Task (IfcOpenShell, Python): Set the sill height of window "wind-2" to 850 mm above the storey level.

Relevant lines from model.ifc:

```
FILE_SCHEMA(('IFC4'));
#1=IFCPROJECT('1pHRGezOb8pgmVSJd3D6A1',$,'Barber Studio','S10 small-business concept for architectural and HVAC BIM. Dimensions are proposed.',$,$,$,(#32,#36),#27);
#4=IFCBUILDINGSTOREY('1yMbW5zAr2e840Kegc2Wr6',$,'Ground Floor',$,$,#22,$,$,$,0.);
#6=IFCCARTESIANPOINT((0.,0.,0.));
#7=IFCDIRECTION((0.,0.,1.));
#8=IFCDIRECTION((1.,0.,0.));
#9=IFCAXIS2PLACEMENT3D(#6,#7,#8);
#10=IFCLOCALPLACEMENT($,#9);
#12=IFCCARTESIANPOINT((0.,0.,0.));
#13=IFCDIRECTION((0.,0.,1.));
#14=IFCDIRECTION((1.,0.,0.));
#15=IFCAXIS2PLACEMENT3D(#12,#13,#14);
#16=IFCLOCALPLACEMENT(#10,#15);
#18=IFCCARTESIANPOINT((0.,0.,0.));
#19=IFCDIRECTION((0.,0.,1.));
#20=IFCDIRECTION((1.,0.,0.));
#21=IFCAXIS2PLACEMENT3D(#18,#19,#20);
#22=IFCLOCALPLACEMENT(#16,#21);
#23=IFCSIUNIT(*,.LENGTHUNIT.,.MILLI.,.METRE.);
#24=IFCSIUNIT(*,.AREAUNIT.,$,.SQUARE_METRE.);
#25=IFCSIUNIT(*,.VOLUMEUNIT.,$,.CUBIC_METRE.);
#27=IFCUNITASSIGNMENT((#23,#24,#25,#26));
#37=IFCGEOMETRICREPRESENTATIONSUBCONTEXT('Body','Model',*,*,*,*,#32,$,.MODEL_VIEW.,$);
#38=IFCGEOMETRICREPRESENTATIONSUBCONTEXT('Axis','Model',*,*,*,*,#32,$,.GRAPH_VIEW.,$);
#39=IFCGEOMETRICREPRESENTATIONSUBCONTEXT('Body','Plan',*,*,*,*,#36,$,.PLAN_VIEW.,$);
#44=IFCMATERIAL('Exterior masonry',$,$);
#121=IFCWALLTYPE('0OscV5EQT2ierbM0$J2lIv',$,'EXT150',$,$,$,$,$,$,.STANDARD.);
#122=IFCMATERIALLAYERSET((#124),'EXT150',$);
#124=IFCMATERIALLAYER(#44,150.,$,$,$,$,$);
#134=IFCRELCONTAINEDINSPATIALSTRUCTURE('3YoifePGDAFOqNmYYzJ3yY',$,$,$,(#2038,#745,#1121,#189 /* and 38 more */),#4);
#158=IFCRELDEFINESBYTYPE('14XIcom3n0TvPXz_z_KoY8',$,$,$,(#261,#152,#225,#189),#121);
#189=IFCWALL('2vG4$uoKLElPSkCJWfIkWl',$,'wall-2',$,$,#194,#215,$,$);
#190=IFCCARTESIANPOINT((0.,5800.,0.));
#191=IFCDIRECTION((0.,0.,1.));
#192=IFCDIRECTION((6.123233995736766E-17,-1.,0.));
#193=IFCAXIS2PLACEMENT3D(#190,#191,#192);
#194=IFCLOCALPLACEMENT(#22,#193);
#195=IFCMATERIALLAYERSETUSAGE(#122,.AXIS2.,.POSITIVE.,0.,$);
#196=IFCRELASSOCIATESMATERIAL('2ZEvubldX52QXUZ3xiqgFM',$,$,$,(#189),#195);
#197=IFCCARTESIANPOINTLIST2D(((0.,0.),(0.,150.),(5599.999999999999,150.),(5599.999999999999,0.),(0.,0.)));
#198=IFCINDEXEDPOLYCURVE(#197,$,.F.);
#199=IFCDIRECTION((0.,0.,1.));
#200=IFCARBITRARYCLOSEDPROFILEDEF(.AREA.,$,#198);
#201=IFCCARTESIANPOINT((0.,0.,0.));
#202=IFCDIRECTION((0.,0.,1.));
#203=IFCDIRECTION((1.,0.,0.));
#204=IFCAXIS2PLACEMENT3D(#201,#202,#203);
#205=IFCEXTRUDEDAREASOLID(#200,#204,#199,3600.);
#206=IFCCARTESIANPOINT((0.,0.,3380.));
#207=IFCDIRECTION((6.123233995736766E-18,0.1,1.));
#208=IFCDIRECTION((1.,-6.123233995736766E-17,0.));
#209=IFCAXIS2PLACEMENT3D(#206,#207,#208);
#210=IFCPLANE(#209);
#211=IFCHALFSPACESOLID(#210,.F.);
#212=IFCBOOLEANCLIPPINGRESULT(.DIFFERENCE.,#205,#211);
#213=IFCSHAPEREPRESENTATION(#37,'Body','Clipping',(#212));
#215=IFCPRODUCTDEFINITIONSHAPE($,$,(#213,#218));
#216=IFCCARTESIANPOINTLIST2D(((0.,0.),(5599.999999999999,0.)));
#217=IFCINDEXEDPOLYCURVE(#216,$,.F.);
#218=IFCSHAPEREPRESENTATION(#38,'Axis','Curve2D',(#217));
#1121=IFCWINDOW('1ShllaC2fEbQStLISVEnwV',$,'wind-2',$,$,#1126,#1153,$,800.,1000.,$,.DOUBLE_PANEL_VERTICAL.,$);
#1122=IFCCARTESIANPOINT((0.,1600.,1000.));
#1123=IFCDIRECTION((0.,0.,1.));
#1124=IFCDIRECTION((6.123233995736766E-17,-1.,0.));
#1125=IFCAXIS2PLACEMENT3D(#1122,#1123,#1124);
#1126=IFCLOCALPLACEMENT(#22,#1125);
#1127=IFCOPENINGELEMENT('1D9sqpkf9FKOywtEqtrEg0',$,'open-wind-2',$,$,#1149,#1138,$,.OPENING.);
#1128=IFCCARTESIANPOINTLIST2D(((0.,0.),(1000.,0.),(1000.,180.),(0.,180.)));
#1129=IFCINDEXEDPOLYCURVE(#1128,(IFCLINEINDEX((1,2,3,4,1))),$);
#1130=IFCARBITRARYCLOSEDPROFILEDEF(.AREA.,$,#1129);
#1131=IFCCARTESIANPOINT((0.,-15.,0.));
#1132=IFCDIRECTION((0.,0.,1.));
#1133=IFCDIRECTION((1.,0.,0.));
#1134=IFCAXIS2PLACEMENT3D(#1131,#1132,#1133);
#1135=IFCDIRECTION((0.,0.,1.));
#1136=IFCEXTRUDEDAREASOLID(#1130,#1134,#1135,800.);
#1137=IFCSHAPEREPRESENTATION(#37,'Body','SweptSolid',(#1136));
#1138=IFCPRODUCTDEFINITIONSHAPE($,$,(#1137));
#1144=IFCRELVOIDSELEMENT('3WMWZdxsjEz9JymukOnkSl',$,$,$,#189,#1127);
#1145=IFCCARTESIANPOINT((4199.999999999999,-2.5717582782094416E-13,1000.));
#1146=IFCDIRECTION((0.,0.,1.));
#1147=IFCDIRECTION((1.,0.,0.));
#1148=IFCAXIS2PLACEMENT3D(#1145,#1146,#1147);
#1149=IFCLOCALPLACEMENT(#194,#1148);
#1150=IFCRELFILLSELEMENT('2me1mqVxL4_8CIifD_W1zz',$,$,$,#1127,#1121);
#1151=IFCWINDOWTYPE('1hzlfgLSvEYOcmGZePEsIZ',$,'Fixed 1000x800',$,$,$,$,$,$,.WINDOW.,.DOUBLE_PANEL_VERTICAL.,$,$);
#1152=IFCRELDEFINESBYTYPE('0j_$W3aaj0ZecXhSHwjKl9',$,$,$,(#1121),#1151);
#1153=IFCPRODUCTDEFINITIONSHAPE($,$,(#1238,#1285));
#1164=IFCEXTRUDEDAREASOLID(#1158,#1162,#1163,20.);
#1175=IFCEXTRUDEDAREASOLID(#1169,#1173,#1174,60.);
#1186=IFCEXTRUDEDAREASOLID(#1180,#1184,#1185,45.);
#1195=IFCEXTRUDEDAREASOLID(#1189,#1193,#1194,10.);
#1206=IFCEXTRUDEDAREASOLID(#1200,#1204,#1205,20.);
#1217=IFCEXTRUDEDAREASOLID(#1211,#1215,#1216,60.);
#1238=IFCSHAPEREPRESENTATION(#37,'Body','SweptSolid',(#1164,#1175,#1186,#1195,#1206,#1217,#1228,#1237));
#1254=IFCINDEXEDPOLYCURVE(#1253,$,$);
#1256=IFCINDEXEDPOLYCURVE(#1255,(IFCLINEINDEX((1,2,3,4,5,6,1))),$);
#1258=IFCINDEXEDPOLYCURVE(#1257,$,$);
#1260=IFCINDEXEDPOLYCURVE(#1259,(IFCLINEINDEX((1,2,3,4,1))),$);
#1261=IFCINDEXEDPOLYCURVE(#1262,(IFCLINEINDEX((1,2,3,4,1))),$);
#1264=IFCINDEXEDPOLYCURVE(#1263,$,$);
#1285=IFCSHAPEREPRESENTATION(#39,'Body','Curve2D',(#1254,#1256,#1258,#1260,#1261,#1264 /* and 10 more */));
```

```python
import numpy as np
import ifcopenshell
import ifcopenshell.api.geometry
import ifcopenshell.geom
import ifcopenshell.util.element
import ifcopenshell.util.placement
import ifcopenshell.util.shape
import ifcopenshell.util.unit

model = ifcopenshell.open("model.ifc")
unit_scale = ifcopenshell.util.unit.calculate_unit_scale(model)

window = model.by_guid("1ShllaC2fEbQStLISVEnwV")
opening = window.FillsVoids[0].RelatingOpeningElement
storey = ifcopenshell.util.element.get_container(window, ifc_class="IfcBuildingStorey")
level = ifcopenshell.util.placement.get_local_placement(storey.ObjectPlacement)[2, 3]

# The opening's origin need not be at the sill, so measure its lowest point.
shape = ifcopenshell.geom.create_shape(ifcopenshell.geom.settings(), opening)
bottom = ifcopenshell.util.shape.get_shape_bottom_elevation(shape, shape.geometry) / unit_scale
dz = level + 850.0 - bottom

shift = np.array([0.0, 0.0, dz])
# The window is not placed relative to its opening, so move both.
for product in (opening, window):
    matrix = ifcopenshell.util.placement.get_local_placement(product.ObjectPlacement)
    matrix[:3, 3] += shift
    ifcopenshell.api.geometry.edit_object_placement(model, product=product, matrix=matrix, is_si=False)

print(f"moved by {dz * unit_scale:+.3f} m")

model.write("model_v2.ifc")
```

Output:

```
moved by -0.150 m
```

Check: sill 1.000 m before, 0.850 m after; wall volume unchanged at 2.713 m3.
